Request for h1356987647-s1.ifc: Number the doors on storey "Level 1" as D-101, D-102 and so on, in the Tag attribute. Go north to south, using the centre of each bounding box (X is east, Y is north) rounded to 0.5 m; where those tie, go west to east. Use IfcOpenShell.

First a look at what the model holds.

```python
import ifcopenshell
import ifcopenshell.util.element
import ifcopenshell.util.placement

model = ifcopenshell.open("h1356987647-s1.ifc")
print(model.schema)
storey = next(s for s in model.by_type("IfcBuildingStorey") if s.Name == "Level 1")
doors = [e for e in ifcopenshell.util.element.get_decomposition(storey) if e.is_a("IfcDoor")]
for e in sorted(doors, key=lambda e: e.id()):
    origin = ifcopenshell.util.placement.get_local_placement(e.ObjectPlacement)[:3, 3]
    print(e.id(), e.Tag, e.Name, origin.round(2) + 0.0, sep=" | ")
```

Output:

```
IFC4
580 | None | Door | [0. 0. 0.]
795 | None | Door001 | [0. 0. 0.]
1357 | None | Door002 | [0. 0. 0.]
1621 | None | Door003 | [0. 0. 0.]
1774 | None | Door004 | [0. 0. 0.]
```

```python
import ifcopenshell
import ifcopenshell.geom
import ifcopenshell.util.element
import ifcopenshell.util.shape

model = ifcopenshell.open("h1356987647-s1.ifc")
settings = ifcopenshell.geom.settings()
settings.set("use-world-coords", True)


def centre(element):
    shape = ifcopenshell.geom.create_shape(settings, element)
    return ifcopenshell.util.shape.get_bbox_centroid(shape.geometry)


storey = next(s for s in model.by_type("IfcBuildingStorey") if s.Name == "Level 1")
doors = [e for e in ifcopenshell.util.element.get_decomposition(storey) if e.is_a("IfcDoor")]

# Insertion points can sit at a corner or the storey origin, so sort by the geometry (in metres).
centres = {e: centre(e) for e in doors}
doors.sort(key=lambda e: (-round(centres[e][1] / 0.5), centres[e][0]))

for i, e in enumerate(doors, start=1):
    number = f"D-1{i:02d}"
    e.Tag = number
    print(e.id(), number)

model.write("h1356987647-s1_edited.ifc")
```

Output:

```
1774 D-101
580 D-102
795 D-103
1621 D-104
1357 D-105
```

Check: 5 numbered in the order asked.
